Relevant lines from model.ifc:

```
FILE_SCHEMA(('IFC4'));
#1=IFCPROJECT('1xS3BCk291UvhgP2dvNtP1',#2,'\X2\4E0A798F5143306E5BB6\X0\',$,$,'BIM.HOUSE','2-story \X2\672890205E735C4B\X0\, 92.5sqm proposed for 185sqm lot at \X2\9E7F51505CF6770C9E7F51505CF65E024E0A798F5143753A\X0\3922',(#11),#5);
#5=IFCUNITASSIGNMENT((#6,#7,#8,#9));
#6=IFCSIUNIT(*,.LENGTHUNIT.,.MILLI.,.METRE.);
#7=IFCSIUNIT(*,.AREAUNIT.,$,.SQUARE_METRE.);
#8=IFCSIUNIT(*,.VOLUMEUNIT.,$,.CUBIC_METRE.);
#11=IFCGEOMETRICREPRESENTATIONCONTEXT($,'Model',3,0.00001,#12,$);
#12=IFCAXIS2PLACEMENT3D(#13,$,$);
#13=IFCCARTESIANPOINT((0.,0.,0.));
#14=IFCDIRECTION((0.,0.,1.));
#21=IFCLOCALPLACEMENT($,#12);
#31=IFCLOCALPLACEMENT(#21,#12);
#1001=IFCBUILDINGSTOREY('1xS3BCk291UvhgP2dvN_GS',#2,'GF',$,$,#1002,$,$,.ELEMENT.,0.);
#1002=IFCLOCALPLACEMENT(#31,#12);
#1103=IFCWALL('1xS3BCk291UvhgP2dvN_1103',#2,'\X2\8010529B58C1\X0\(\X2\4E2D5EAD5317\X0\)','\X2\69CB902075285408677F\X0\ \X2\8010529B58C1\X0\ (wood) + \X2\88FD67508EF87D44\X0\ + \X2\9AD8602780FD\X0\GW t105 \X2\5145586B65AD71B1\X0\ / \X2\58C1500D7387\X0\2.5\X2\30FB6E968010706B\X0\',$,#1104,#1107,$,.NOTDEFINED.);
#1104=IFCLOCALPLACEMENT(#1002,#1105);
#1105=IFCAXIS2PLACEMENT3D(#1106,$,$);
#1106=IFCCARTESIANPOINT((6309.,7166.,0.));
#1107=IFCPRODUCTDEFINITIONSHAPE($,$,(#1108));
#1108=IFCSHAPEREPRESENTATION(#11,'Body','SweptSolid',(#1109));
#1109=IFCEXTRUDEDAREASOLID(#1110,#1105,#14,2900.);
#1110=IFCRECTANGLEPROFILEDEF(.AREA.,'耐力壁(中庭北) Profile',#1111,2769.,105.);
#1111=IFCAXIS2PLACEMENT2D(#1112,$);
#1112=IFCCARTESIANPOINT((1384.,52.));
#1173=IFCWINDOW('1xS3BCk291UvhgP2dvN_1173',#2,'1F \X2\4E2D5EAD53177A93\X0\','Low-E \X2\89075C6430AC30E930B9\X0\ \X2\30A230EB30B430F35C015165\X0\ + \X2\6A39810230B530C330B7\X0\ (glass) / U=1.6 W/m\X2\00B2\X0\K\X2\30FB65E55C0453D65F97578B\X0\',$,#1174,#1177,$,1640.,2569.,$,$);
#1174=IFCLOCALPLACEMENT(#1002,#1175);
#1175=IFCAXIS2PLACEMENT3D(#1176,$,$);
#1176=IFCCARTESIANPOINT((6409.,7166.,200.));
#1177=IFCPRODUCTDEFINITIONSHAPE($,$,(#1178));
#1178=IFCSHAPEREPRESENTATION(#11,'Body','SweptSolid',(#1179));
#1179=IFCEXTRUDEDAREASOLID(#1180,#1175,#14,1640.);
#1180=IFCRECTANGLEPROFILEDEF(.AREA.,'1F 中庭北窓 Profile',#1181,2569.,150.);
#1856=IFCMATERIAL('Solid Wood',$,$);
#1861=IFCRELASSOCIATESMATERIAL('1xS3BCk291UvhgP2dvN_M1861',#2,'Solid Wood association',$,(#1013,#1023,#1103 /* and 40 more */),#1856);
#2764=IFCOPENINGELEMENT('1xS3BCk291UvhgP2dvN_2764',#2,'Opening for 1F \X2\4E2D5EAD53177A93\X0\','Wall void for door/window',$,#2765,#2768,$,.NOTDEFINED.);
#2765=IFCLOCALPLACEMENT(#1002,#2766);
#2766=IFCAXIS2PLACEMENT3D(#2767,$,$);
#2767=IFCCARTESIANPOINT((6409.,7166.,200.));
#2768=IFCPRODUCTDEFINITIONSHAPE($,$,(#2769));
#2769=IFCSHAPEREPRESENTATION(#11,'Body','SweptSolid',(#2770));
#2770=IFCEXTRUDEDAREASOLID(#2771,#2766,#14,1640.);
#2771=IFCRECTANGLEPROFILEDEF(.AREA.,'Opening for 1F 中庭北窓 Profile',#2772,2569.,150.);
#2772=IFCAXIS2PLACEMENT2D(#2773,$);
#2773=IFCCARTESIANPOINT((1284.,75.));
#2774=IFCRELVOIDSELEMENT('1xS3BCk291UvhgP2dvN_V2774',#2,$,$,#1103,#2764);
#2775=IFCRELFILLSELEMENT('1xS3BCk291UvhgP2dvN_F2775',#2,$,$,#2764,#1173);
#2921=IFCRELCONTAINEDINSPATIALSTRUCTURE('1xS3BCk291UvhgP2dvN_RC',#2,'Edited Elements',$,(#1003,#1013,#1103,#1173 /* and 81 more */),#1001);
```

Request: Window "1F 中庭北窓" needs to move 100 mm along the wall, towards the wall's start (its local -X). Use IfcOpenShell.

```python
import ifcopenshell
import ifcopenshell.api.geometry
import ifcopenshell.util.placement
import ifcopenshell.util.unit

model = ifcopenshell.open("model.ifc")
unit_scale = ifcopenshell.util.unit.calculate_unit_scale(model)

window = model.by_guid("1xS3BCk291UvhgP2dvN_1173")
opening = window.FillsVoids[0].RelatingOpeningElement
wall = opening.VoidsElements[0].RelatingBuildingElement

wall_matrix = ifcopenshell.util.placement.get_local_placement(wall.ObjectPlacement)
shift = wall_matrix[:3, 0] * -0.1 / unit_scale
before = ifcopenshell.util.placement.get_local_placement(window.ObjectPlacement)[:3, 3].copy()

# The window is not placed relative to its opening, so move both.
for product in (opening, window):
    matrix = ifcopenshell.util.placement.get_local_placement(product.ObjectPlacement)
    matrix[:3, 3] += shift
    ifcopenshell.api.geometry.edit_object_placement(model, product=product, matrix=matrix, is_si=False)

after = ifcopenshell.util.placement.get_local_placement(window.ObjectPlacement)[:3, 3]
print("window moved by", (after - before).round(3) + 0.0)

model.write("model_v2.ifc")
```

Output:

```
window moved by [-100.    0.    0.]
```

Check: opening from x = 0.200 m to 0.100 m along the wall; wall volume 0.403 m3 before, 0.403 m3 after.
